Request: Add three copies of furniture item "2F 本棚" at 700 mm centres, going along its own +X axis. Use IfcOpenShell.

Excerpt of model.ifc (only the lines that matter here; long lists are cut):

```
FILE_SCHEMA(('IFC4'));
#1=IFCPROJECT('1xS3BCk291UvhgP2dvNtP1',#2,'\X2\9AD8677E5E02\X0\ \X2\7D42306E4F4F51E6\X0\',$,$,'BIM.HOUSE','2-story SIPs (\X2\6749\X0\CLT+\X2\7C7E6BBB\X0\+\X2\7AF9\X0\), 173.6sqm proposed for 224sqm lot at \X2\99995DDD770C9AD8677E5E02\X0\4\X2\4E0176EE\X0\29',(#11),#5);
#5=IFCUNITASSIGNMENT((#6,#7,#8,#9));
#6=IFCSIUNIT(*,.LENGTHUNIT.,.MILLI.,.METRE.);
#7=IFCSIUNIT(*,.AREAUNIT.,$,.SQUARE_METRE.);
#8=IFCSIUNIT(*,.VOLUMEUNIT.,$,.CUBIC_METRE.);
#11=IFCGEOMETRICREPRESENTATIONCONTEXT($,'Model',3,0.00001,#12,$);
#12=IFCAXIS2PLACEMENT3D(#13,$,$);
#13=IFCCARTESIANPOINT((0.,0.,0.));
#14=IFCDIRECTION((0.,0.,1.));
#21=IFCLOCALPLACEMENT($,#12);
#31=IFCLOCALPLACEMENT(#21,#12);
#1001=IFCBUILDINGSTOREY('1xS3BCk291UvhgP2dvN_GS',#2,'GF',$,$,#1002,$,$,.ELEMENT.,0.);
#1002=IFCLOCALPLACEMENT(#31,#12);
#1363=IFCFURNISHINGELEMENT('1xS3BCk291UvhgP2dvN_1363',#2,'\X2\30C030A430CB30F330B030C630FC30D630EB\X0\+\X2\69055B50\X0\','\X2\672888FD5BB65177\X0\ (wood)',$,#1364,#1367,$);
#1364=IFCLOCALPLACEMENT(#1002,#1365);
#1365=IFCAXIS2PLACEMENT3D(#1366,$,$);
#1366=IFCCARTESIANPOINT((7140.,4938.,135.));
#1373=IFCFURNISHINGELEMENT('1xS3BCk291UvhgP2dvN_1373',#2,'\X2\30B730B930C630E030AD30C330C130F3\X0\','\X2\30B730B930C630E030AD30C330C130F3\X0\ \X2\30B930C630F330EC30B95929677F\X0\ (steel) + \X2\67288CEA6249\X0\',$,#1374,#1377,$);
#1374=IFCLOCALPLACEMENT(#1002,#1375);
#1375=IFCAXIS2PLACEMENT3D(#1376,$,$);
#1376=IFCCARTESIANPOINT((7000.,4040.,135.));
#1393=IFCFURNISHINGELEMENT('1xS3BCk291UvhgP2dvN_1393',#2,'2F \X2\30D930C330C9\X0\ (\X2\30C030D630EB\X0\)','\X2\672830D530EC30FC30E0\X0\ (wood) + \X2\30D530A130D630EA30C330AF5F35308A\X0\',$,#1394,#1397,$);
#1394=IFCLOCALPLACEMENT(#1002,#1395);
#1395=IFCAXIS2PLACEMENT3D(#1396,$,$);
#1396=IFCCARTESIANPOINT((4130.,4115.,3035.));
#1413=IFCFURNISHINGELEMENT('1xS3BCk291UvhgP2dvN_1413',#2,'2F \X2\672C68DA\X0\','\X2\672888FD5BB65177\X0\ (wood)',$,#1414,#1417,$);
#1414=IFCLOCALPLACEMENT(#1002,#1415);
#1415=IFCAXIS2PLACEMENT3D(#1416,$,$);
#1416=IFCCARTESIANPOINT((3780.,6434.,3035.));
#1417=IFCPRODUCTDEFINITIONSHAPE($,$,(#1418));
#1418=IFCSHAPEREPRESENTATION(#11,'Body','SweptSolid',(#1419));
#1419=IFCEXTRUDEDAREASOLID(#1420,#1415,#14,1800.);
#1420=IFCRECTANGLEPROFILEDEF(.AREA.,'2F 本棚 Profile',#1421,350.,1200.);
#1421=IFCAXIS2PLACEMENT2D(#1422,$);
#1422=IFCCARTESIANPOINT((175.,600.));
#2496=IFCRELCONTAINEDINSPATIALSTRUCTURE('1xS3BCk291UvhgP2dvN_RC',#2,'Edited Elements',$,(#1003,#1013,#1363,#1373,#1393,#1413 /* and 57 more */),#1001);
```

```python
import ifcopenshell
import ifcopenshell.api.geometry
import ifcopenshell.api.root
import ifcopenshell.util.element
import ifcopenshell.util.placement
import ifcopenshell.util.unit

model = ifcopenshell.open("model.ifc")
unit_scale = ifcopenshell.util.unit.calculate_unit_scale(model)


def reuse_history(source, copy):
    """copy_class also copies each property set's owner history, people and application; keep the originals."""
    for rel in copy.IsDefinedBy:
        if rel.is_a("IfcRelDefinesByProperties") and (history := rel.RelatingPropertyDefinition.OwnerHistory):
            rel.RelatingPropertyDefinition.OwnerHistory = source.OwnerHistory
            ifcopenshell.util.element.remove_deep2(model, history)


source = model.by_guid("1xS3BCk291UvhgP2dvN_1413")
base = ifcopenshell.util.placement.get_local_placement(source.ObjectPlacement)
step = base[:3, 0] * 0.7 / unit_scale

for i in range(1, 4):
    copy = ifcopenshell.api.root.copy_class(model, product=source)
    copy.Representation = ifcopenshell.util.element.copy_deep(
        model, source.Representation, exclude=["IfcGeometricRepresentationContext", "IfcRepresentationMap"]
    )
    reuse_history(source, copy)
    matrix = base.copy()
    matrix[:3, 3] += i * step
    print("added at", matrix[:3, 3].round(3) + 0.0)
    ifcopenshell.api.geometry.edit_object_placement(model, product=copy, matrix=matrix, is_si=False)

model.write("model_rev.ifc")
```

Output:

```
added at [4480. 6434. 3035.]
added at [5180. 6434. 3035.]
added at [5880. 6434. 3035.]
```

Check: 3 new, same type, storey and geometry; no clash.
